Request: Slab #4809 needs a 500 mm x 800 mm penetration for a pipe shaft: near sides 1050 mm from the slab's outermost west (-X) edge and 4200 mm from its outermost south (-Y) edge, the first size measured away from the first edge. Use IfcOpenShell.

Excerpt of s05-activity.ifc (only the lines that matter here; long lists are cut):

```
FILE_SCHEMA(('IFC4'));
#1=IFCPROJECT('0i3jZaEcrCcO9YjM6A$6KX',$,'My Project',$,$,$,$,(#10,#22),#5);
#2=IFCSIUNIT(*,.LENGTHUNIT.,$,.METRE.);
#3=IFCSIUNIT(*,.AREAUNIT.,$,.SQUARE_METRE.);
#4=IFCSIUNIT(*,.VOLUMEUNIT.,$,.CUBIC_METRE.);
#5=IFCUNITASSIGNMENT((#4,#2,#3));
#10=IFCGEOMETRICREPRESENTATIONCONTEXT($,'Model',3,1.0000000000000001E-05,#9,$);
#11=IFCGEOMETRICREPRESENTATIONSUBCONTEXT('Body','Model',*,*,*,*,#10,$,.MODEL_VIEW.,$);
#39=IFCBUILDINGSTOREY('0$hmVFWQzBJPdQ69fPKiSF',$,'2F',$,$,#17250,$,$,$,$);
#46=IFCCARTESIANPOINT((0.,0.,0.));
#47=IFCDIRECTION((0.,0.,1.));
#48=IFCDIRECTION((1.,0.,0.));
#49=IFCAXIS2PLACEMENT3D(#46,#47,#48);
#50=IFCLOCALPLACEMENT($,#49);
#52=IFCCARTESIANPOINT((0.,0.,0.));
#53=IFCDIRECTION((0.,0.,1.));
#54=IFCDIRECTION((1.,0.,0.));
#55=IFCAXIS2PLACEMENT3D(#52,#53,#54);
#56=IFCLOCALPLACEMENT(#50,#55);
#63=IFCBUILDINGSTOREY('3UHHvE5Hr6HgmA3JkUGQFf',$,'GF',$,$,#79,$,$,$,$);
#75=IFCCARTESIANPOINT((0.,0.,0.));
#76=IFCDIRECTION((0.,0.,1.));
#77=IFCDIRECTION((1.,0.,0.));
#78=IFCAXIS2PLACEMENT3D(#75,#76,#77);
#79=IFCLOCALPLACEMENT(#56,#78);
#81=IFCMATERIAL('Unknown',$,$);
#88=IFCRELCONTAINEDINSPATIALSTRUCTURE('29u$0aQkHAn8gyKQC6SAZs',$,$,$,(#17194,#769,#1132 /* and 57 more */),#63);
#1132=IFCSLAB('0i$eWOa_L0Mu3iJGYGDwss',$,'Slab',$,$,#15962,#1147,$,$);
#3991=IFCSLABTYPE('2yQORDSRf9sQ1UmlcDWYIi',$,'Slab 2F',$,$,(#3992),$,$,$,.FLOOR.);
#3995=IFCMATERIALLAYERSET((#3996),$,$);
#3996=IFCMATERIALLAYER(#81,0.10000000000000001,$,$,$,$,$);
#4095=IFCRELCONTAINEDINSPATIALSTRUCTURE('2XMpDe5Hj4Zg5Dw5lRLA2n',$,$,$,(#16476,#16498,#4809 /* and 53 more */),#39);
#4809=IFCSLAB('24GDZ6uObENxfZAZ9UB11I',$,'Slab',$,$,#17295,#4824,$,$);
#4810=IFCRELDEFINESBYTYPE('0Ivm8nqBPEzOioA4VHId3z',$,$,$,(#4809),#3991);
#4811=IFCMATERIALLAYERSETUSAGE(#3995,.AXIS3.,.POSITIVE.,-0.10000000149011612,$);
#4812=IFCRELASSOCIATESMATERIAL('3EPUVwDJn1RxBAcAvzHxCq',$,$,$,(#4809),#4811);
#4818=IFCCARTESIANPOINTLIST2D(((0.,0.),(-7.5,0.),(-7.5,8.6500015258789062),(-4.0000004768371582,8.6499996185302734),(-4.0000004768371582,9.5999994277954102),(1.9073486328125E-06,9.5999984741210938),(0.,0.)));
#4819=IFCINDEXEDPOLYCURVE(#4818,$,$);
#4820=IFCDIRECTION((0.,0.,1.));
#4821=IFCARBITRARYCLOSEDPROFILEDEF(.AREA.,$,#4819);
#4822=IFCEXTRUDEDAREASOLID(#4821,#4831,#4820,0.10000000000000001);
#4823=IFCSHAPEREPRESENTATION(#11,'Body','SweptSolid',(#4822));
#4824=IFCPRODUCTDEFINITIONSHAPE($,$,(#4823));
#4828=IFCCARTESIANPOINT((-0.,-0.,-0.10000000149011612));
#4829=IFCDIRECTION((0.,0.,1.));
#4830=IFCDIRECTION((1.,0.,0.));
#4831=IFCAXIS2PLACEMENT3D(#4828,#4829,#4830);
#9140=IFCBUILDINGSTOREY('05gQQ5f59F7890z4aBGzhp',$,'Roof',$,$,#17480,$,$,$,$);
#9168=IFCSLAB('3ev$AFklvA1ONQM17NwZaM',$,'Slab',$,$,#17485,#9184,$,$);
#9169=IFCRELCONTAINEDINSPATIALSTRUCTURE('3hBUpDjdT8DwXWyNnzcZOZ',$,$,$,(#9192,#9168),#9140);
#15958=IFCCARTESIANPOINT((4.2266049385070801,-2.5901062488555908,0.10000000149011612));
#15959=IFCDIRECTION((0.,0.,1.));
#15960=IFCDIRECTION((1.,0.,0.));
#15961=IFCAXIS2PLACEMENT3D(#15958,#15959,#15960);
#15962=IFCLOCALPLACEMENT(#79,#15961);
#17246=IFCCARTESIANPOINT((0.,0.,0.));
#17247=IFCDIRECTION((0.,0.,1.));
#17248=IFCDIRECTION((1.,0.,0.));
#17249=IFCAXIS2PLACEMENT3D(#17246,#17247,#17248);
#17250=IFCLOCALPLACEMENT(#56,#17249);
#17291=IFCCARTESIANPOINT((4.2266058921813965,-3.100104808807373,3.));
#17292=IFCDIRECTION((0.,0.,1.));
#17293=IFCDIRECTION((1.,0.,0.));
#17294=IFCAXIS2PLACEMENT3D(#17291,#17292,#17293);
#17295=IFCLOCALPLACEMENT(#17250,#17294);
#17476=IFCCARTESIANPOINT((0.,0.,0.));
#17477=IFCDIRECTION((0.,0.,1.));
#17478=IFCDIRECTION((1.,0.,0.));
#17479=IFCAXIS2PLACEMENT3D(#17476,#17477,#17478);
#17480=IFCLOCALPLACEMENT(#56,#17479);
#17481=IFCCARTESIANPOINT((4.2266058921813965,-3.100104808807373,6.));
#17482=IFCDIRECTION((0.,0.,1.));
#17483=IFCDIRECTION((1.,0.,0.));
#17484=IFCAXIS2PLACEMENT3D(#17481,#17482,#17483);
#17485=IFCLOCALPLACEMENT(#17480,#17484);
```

```python
import numpy as np
import ifcopenshell
import ifcopenshell.api.feature
import ifcopenshell.api.geometry
import ifcopenshell.api.root
import ifcopenshell.geom
import ifcopenshell.util.placement
import ifcopenshell.util.representation
import ifcopenshell.util.shape
import ifcopenshell.util.unit

model = ifcopenshell.open("s05-activity.ifc")
unit_scale = ifcopenshell.util.unit.calculate_unit_scale(model)
settings = ifcopenshell.geom.settings()


def volume(element):
    """Net volume in cubic metres, openings subtracted."""
    shape = ifcopenshell.geom.create_shape(settings, element)
    return ifcopenshell.util.shape.get_volume(shape.geometry)


slab = model.by_guid("24GDZ6uObENxfZAZ9UB11I")
before = volume(slab)

# Extent in the slab's own axes, in metres. The edges named are its -X and -Y sides.
slab_shape = ifcopenshell.geom.create_shape(settings, slab)
vertices = ifcopenshell.util.shape.get_vertices(slab_shape.geometry)
x_min, y_min, bottom = vertices.min(axis=0)
top = vertices[:, 2].max()

opening = ifcopenshell.api.root.create_entity(model, ifc_class="IfcOpeningElement", name="Pipe shaft opening", predefined_type="OPENING")
context = ifcopenshell.util.representation.get_context(model, "Model", "Body", "MODEL_VIEW")
width, depth = 0.5, 0.8
outline = [(0.0, 0.0), (width, 0.0), (width, depth), (0.0, depth), (0.0, 0.0)]
# Overshoot both faces by 50 mm so the cut is clean.
shape = ifcopenshell.api.geometry.add_slab_representation(
    model, context=context, depth=top - bottom + 0.1, polyline=outline
)
ifcopenshell.api.geometry.assign_representation(model, product=opening, representation=shape)

matrix = ifcopenshell.util.placement.get_local_placement(slab.ObjectPlacement)
matrix[:, 3] = matrix @ np.append(np.array([x_min + 1.05, y_min + 4.2, bottom - 0.05]) / unit_scale, 1.0)
ifcopenshell.api.geometry.edit_object_placement(model, product=opening, matrix=matrix, is_si=False)
ifcopenshell.api.feature.add_feature(model, feature=opening, element=slab)

after = volume(slab)

print(f"slab volume {before:.3f} -> {after:.3f} m3")

model.write("s05-activity_edited.ifc")
```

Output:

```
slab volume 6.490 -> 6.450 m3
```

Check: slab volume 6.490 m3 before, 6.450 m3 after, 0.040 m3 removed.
